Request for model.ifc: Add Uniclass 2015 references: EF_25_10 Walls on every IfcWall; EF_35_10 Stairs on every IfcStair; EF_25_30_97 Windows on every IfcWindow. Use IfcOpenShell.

First a look at what the model holds.

```python
import ifcopenshell

model = ifcopenshell.open("model.ifc")
print(model.schema)
print("classifications:", [c.Name for c in model.by_type("IfcClassification")])
for ifc_class in ("IfcDoor", "IfcRoof", "IfcStair", "IfcWall", "IfcWindow"):
    print(ifc_class, len(model.by_type(ifc_class)))
```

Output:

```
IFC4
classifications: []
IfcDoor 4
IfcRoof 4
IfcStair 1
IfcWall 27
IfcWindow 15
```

```python
import ifcopenshell
import ifcopenshell.api.classification

model = ifcopenshell.open("model.ifc")

system = ifcopenshell.api.classification.add_classification(model, classification="Uniclass 2015")

codes = {
    "IfcWall": ("EF_25_10", "Walls"),
    "IfcStair": ("EF_35_10", "Stairs"),
    "IfcWindow": ("EF_25_30_97", "Windows"),
}
for ifc_class, (code, name) in codes.items():
    products = model.by_type(ifc_class)
    ifcopenshell.api.classification.add_reference(
        model, products=products, classification=system, identification=code, name=name
    )
    print(code, len(products))

model.write("model_v2.ifc")
```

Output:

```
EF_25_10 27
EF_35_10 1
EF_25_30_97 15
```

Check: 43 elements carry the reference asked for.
